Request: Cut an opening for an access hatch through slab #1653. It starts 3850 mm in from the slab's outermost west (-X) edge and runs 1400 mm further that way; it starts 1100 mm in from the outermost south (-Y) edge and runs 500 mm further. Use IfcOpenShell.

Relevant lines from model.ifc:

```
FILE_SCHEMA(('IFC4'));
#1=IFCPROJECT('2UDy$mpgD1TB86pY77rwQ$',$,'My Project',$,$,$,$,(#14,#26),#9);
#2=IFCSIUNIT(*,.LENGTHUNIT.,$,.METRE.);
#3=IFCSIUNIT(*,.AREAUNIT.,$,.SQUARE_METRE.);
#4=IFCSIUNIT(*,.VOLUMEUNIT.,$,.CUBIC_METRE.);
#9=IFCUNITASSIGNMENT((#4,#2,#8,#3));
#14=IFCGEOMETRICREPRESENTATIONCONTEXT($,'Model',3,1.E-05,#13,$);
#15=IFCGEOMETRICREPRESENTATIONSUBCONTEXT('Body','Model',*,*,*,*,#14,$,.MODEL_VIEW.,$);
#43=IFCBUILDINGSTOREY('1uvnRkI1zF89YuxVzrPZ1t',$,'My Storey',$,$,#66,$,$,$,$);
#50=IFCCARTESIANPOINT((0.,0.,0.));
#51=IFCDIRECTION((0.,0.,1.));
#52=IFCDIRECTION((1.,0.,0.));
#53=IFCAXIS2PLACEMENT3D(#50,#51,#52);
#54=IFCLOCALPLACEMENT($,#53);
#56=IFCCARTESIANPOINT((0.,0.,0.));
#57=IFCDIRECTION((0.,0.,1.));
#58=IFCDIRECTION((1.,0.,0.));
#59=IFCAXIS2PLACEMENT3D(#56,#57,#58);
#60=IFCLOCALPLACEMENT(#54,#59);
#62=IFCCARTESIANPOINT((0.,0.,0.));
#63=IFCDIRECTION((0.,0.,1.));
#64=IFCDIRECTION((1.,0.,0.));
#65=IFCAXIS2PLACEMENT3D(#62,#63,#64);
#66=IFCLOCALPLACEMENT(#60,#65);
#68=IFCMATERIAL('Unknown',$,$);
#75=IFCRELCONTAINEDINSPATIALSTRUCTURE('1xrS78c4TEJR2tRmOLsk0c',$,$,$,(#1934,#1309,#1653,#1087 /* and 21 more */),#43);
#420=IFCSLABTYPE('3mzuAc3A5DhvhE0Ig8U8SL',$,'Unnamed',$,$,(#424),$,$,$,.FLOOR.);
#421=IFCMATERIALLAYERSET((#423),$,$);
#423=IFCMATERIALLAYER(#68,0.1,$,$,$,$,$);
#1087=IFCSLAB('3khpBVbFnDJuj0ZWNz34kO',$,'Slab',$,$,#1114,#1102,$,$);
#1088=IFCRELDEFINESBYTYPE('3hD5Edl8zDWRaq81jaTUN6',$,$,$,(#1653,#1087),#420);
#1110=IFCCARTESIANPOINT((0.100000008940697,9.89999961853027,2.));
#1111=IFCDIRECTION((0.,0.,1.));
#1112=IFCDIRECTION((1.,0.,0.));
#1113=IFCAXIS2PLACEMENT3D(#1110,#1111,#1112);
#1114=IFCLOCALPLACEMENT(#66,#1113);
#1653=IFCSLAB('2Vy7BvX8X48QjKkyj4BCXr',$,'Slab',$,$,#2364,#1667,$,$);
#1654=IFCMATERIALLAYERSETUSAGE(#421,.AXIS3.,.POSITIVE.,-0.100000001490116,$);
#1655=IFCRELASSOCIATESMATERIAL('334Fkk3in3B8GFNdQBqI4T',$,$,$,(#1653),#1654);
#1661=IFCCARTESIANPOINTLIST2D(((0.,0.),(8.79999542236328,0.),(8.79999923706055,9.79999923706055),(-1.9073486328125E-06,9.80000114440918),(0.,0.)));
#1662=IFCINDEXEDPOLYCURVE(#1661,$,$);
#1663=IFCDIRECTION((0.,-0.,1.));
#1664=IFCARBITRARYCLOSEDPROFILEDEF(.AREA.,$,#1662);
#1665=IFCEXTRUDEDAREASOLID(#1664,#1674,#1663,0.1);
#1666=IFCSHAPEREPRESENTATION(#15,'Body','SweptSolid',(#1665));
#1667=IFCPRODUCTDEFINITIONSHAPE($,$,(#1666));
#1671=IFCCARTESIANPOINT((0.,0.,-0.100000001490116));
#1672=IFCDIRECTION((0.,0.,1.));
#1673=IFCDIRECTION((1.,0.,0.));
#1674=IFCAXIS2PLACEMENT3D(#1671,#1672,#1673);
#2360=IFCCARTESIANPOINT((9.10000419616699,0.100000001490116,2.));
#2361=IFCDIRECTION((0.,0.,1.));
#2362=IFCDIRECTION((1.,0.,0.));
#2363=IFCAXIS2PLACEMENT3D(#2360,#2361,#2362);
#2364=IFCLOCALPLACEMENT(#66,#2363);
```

```python
import numpy as np
import ifcopenshell
import ifcopenshell.api.feature
import ifcopenshell.api.geometry
import ifcopenshell.api.root
import ifcopenshell.geom
import ifcopenshell.util.placement
import ifcopenshell.util.representation
import ifcopenshell.util.shape
import ifcopenshell.util.unit

model = ifcopenshell.open("model.ifc")
unit_scale = ifcopenshell.util.unit.calculate_unit_scale(model)
settings = ifcopenshell.geom.settings()


def volume(element):
    """Net volume in cubic metres, openings subtracted."""
    shape = ifcopenshell.geom.create_shape(settings, element)
    return ifcopenshell.util.shape.get_volume(shape.geometry)


slab = model.by_guid("2Vy7BvX8X48QjKkyj4BCXr")
before = volume(slab)

# Extent in the slab's own axes, in metres. The edges named are its -X and -Y sides.
slab_shape = ifcopenshell.geom.create_shape(settings, slab)
vertices = ifcopenshell.util.shape.get_vertices(slab_shape.geometry)
x_min, y_min, bottom = vertices.min(axis=0)
top = vertices[:, 2].max()

opening = ifcopenshell.api.root.create_entity(model, ifc_class="IfcOpeningElement", name="Access hatch opening", predefined_type="OPENING")
context = ifcopenshell.util.representation.get_context(model, "Model", "Body", "MODEL_VIEW")
width, depth = 1.4, 0.5
outline = [(0.0, 0.0), (width, 0.0), (width, depth), (0.0, depth), (0.0, 0.0)]
# Overshoot both faces by 50 mm so the cut is clean.
shape = ifcopenshell.api.geometry.add_slab_representation(
    model, context=context, depth=top - bottom + 0.1, polyline=outline
)
ifcopenshell.api.geometry.assign_representation(model, product=opening, representation=shape)

matrix = ifcopenshell.util.placement.get_local_placement(slab.ObjectPlacement)
matrix[:, 3] = matrix @ np.append(np.array([x_min + 3.85, y_min + 1.1, bottom - 0.05]) / unit_scale, 1.0)
ifcopenshell.api.geometry.edit_object_placement(model, product=opening, matrix=matrix, is_si=False)
ifcopenshell.api.feature.add_feature(model, feature=opening, element=slab)

after = volume(slab)

print(f"slab volume {before:.3f} -> {after:.3f} m3")

model.write("model_rev.ifc")
```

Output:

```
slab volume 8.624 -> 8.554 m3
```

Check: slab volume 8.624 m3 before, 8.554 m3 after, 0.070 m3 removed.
